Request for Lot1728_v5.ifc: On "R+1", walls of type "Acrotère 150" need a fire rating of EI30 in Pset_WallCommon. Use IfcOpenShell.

First a look at what the model holds.

```python
import ifcopenshell
import ifcopenshell.util.element

model = ifcopenshell.open("Lot1728_v5.ifc")
print(model.schema)
storey = next(s for s in model.by_type("IfcBuildingStorey") if s.Name == "R+1")
walls = [e for e in ifcopenshell.util.element.get_decomposition(storey) if e.is_a("IfcWall")]
seen = {}
for e in walls:
    element_type = ifcopenshell.util.element.get_type(e)
    key = (element_type.Name if element_type != e and element_type else None, ifcopenshell.util.element.get_pset(e, "Pset_WallCommon", "FireRating"))
    seen[key] = seen.get(key, 0) + 1
for (name, value), count in sorted(seen.items(), key=str):
    print(count, "x", name, "|", value)
```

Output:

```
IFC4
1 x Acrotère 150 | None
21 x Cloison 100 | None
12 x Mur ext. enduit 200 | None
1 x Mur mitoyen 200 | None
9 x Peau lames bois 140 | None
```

```python
import ifcopenshell
import ifcopenshell.api.pset
import ifcopenshell.util.element

model = ifcopenshell.open("Lot1728_v5.ifc")

storey = next(s for s in model.by_type("IfcBuildingStorey") if s.Name == "R+1")
walls = [e for e in ifcopenshell.util.element.get_decomposition(storey) if e.is_a("IfcWall")]

count = 0
for e in walls:
    element_type = ifcopenshell.util.element.get_type(e)
    if element_type in (None, e) or element_type.Name != "Acrotère 150":
        continue
    # add_pset returns the element's existing set when there is one.
    pset = ifcopenshell.api.pset.add_pset(model, product=e, name="Pset_WallCommon")
    ifcopenshell.api.pset.edit_pset(model, pset=pset, properties={"FireRating": "EI30"})
    count += 1

print(count, "walls updated")

model.write("Lot1728_v5_rev.ifc")
```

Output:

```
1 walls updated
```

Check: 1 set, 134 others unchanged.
